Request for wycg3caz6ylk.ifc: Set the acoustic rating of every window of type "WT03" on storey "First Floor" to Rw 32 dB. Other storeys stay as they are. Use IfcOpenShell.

First a look at what the model holds.

```python
import ifcopenshell
import ifcopenshell.util.element

model = ifcopenshell.open("wycg3caz6ylk.ifc")
print(model.schema)
storey = next(s for s in model.by_type("IfcBuildingStorey") if s.Name == "First Floor")
windows = [e for e in ifcopenshell.util.element.get_decomposition(storey) if e.is_a("IfcWindow")]
seen = {}
for e in windows:
    element_type = ifcopenshell.util.element.get_type(e)
    key = (element_type.Name if element_type != e and element_type else None, ifcopenshell.util.element.get_pset(e, "Pset_WindowCommon", "AcousticRating"))
    seen[key] = seen.get(key, 0) + 1
for (name, value), count in sorted(seen.items(), key=str):
    print(count, "x", name, "|", value)
```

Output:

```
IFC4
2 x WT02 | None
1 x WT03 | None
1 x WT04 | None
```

```python
import ifcopenshell
import ifcopenshell.api.pset
import ifcopenshell.util.element

model = ifcopenshell.open("wycg3caz6ylk.ifc")

storey = next(s for s in model.by_type("IfcBuildingStorey") if s.Name == "First Floor")
windows = [e for e in ifcopenshell.util.element.get_decomposition(storey) if e.is_a("IfcWindow")]

count = 0
for e in windows:
    element_type = ifcopenshell.util.element.get_type(e)
    if element_type in (None, e) or element_type.Name != "WT03":
        continue
    # add_pset returns the element's existing set when there is one.
    pset = ifcopenshell.api.pset.add_pset(model, product=e, name="Pset_WindowCommon")
    ifcopenshell.api.pset.edit_pset(model, pset=pset, properties={"AcousticRating": "Rw 32 dB"})
    count += 1

print(count, "windows updated")

model.write("wycg3caz6ylk_edited.ifc")
```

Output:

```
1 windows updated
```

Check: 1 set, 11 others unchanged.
